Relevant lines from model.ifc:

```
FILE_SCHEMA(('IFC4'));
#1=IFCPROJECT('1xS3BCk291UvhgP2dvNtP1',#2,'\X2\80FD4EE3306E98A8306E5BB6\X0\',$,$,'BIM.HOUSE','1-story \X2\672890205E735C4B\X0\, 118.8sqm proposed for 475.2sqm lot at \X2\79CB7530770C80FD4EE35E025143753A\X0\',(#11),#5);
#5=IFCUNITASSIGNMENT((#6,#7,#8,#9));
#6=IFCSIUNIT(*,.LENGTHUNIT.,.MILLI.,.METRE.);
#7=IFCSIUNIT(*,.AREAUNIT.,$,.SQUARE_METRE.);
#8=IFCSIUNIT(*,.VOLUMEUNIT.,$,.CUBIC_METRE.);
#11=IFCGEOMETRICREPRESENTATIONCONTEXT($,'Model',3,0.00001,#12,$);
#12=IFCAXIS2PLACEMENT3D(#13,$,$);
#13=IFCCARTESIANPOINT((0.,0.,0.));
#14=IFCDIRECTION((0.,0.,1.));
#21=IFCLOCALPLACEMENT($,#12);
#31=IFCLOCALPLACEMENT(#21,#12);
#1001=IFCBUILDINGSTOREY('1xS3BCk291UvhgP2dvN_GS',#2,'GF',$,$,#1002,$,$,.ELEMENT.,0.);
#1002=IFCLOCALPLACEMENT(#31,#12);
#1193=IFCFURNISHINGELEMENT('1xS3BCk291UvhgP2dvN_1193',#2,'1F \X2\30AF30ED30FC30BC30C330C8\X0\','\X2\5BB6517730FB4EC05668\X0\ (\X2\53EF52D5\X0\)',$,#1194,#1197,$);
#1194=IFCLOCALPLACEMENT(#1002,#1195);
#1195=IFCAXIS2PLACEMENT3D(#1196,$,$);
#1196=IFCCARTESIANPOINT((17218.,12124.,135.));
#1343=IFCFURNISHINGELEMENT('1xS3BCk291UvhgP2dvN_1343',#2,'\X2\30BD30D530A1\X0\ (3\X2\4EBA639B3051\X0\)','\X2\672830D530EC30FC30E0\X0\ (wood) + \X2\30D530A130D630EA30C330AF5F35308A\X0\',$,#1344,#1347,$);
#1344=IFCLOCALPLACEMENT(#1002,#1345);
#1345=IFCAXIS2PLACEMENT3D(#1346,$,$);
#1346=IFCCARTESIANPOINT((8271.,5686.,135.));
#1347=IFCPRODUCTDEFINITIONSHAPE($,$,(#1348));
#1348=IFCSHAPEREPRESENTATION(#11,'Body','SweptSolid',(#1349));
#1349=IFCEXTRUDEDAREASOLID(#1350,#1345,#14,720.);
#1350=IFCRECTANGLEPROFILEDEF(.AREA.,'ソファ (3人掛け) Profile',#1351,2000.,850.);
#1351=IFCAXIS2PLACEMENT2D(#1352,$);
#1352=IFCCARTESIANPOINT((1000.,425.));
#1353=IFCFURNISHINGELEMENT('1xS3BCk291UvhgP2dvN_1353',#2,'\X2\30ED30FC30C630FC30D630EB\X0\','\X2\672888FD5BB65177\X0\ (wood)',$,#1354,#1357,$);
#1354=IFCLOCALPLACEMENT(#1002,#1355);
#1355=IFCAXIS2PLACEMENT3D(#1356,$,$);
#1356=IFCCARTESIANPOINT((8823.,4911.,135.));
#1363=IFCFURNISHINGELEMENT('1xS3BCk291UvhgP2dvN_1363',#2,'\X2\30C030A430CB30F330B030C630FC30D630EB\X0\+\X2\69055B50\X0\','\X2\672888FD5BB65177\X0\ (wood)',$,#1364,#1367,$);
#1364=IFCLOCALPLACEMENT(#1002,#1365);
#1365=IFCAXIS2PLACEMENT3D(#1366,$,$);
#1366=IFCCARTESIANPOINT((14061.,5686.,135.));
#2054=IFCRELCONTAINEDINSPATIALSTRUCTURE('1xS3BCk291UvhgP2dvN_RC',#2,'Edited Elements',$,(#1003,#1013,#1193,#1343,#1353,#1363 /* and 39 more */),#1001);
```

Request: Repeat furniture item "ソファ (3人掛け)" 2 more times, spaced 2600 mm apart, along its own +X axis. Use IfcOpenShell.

```python
import ifcopenshell
import ifcopenshell.api.geometry
import ifcopenshell.api.root
import ifcopenshell.util.element
import ifcopenshell.util.placement

model = ifcopenshell.open("model.ifc")


def reuse_history(source, copy):
    """copy_class also copies each property set's owner history, people and application; keep the originals."""
    for rel in copy.IsDefinedBy:
        if rel.is_a("IfcRelDefinesByProperties") and (history := rel.RelatingPropertyDefinition.OwnerHistory):
            rel.RelatingPropertyDefinition.OwnerHistory = source.OwnerHistory
            ifcopenshell.util.element.remove_deep2(model, history)


source = model.by_guid("1xS3BCk291UvhgP2dvN_1343")
base = ifcopenshell.util.placement.get_local_placement(source.ObjectPlacement)
step = base[:3, 0] * 2600.0

for i in range(1, 3):
    copy = ifcopenshell.api.root.copy_class(model, product=source)
    copy.Representation = ifcopenshell.util.element.copy_deep(
        model, source.Representation, exclude=["IfcGeometricRepresentationContext", "IfcRepresentationMap"]
    )
    reuse_history(source, copy)
    matrix = base.copy()
    matrix[:3, 3] += i * step
    print("added at", matrix[:3, 3].round(3) + 0.0)
    ifcopenshell.api.geometry.edit_object_placement(model, product=copy, matrix=matrix, is_si=False)

model.write("model_updated.ifc")
```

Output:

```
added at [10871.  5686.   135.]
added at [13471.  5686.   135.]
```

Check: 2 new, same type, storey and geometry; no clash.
